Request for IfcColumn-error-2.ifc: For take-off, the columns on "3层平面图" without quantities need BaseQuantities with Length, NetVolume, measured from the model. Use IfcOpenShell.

First a look at what the model holds.

```python
import ifcopenshell
import ifcopenshell.util.element
import ifcopenshell.util.unit

model = ifcopenshell.open("IfcColumn-error-2.ifc")
print(model.schema)
for unit_type in ("LENGTHUNIT", "AREAUNIT", "VOLUMEUNIT"):
    print(unit_type, ifcopenshell.util.unit.calculate_unit_scale(model, unit_type))
storey = next(s for s in model.by_type("IfcBuildingStorey") if s.Name == "3层平面图")
columns = [e for e in ifcopenshell.util.element.get_decomposition(storey) if e.is_a("IfcColumn")]
for e in sorted(columns, key=lambda e: e.id()):
    print(e.id(), e.is_a(), e.Name, list(ifcopenshell.util.element.get_psets(e, qtos_only=True)), sep=" | ")
```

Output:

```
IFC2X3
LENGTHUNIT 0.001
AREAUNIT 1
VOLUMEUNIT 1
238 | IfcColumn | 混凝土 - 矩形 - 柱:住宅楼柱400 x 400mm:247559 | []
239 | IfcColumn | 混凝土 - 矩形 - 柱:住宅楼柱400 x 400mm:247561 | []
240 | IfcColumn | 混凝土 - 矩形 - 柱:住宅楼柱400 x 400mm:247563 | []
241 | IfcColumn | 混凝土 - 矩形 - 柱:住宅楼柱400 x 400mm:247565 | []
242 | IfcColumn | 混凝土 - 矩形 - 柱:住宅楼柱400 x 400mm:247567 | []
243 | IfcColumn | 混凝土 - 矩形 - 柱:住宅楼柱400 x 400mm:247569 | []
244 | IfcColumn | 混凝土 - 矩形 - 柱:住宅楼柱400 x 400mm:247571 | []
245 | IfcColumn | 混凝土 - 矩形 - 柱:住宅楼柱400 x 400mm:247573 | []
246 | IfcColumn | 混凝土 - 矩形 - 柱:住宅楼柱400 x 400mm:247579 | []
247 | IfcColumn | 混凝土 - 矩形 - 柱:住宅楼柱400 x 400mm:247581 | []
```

```python
import ifcopenshell
import ifcopenshell.api.pset
import ifcopenshell.geom
import ifcopenshell.util.element
import ifcopenshell.util.shape
import ifcopenshell.util.unit

model = ifcopenshell.open("IfcColumn-error-2.ifc")
unit_scale = ifcopenshell.util.unit.calculate_unit_scale(model)
volume_scale = ifcopenshell.util.unit.calculate_unit_scale(model, "VOLUMEUNIT")
settings = ifcopenshell.geom.settings()

storey = next(s for s in model.by_type("IfcBuildingStorey") if s.Name == "3层平面图")
columns = [e for e in ifcopenshell.util.element.get_decomposition(storey) if e.is_a("IfcColumn")]

for e in sorted(columns, key=lambda e: e.id()):
    if ifcopenshell.util.element.get_psets(e, qtos_only=True, should_inherit=False):
        continue
    # Geometry comes back in metres, in the element's own axes.
    shape = ifcopenshell.geom.create_shape(settings, e)
    values = {
        "Length": ifcopenshell.util.shape.get_z(shape.geometry) / unit_scale,
        "NetVolume": ifcopenshell.util.shape.get_volume(shape.geometry) / volume_scale,
    }
    qto = ifcopenshell.api.pset.add_qto(model, product=e, name="BaseQuantities")
    ifcopenshell.api.pset.edit_qto(model, qto=qto, properties=values)
    print(e.id(), {k: round(v, 3) for k, v in values.items()})

model.write("IfcColumn-error-2_edited.ifc")
```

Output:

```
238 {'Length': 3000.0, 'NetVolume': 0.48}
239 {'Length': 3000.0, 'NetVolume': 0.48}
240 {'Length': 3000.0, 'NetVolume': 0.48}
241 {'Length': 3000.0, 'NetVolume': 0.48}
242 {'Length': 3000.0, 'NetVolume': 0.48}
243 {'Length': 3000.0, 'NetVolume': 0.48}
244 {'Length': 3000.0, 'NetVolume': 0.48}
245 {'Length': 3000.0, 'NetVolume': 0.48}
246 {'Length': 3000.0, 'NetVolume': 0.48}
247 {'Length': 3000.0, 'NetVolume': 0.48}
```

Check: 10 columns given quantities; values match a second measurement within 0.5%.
